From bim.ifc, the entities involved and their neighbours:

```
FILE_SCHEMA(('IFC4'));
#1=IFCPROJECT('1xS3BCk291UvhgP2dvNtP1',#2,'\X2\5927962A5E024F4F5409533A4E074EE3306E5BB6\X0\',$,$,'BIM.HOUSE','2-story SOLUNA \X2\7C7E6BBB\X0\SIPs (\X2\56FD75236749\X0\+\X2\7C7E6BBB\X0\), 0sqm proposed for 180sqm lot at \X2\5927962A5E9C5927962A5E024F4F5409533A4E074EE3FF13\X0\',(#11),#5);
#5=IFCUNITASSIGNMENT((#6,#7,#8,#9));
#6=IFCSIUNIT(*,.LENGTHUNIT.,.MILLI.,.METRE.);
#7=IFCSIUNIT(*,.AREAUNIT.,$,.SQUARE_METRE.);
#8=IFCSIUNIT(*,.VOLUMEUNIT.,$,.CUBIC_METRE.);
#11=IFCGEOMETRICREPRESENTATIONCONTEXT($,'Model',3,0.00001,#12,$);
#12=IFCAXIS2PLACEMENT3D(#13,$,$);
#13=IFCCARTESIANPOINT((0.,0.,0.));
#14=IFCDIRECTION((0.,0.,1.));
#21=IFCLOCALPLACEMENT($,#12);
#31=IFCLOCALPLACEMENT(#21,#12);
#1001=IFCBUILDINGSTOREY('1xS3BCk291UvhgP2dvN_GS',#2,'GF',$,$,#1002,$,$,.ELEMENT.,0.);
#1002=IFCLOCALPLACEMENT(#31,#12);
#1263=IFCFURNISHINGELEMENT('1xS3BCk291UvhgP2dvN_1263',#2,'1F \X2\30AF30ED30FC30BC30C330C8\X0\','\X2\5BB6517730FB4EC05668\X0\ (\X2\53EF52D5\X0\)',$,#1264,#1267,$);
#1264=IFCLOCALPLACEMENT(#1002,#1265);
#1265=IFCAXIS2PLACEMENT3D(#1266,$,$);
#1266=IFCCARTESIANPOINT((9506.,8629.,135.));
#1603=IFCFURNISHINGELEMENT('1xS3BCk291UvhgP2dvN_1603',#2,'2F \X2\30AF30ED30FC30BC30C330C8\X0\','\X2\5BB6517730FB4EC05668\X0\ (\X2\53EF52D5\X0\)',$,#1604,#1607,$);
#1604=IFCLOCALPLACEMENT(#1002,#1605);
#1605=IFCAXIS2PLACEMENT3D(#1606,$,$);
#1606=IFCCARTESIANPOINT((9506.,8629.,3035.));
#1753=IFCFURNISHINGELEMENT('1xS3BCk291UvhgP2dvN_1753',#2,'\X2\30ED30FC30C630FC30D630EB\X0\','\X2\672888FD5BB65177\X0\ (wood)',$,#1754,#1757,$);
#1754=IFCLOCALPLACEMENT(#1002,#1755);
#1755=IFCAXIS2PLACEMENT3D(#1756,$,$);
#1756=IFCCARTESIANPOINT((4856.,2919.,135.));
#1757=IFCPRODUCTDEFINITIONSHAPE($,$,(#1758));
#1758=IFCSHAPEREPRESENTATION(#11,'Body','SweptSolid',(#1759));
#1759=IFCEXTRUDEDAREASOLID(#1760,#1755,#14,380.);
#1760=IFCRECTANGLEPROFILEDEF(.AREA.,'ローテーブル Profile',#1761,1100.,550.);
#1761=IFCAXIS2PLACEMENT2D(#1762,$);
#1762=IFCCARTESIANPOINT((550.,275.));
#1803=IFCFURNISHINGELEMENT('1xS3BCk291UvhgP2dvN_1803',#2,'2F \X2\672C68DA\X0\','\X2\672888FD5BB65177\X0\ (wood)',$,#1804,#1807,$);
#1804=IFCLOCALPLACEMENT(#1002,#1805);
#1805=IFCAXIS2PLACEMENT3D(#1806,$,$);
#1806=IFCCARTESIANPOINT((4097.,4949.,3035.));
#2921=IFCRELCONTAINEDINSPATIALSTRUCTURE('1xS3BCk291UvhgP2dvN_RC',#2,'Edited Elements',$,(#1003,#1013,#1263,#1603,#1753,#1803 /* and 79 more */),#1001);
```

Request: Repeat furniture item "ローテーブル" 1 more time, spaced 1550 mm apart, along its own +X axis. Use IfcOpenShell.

```python
import ifcopenshell
import ifcopenshell.api.geometry
import ifcopenshell.api.root
import ifcopenshell.util.element
import ifcopenshell.util.placement

model = ifcopenshell.open("bim.ifc")


def reuse_history(source, copy):
    """copy_class also copies each property set's owner history, people and application; keep the originals."""
    for rel in copy.IsDefinedBy:
        if rel.is_a("IfcRelDefinesByProperties") and (history := rel.RelatingPropertyDefinition.OwnerHistory):
            rel.RelatingPropertyDefinition.OwnerHistory = source.OwnerHistory
            ifcopenshell.util.element.remove_deep2(model, history)


source = model.by_guid("1xS3BCk291UvhgP2dvN_1753")
base = ifcopenshell.util.placement.get_local_placement(source.ObjectPlacement)
step = base[:3, 0] * 1550.0

for i in range(1, 2):
    copy = ifcopenshell.api.root.copy_class(model, product=source)
    copy.Representation = ifcopenshell.util.element.copy_deep(
        model, source.Representation, exclude=["IfcGeometricRepresentationContext", "IfcRepresentationMap"]
    )
    reuse_history(source, copy)
    matrix = base.copy()
    matrix[:3, 3] += i * step
    print("added at", matrix[:3, 3].round(3) + 0.0)
    ifcopenshell.api.geometry.edit_object_placement(model, product=copy, matrix=matrix, is_si=False)

model.write("bim_edited.ifc")
```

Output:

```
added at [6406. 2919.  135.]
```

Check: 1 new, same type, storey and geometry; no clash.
